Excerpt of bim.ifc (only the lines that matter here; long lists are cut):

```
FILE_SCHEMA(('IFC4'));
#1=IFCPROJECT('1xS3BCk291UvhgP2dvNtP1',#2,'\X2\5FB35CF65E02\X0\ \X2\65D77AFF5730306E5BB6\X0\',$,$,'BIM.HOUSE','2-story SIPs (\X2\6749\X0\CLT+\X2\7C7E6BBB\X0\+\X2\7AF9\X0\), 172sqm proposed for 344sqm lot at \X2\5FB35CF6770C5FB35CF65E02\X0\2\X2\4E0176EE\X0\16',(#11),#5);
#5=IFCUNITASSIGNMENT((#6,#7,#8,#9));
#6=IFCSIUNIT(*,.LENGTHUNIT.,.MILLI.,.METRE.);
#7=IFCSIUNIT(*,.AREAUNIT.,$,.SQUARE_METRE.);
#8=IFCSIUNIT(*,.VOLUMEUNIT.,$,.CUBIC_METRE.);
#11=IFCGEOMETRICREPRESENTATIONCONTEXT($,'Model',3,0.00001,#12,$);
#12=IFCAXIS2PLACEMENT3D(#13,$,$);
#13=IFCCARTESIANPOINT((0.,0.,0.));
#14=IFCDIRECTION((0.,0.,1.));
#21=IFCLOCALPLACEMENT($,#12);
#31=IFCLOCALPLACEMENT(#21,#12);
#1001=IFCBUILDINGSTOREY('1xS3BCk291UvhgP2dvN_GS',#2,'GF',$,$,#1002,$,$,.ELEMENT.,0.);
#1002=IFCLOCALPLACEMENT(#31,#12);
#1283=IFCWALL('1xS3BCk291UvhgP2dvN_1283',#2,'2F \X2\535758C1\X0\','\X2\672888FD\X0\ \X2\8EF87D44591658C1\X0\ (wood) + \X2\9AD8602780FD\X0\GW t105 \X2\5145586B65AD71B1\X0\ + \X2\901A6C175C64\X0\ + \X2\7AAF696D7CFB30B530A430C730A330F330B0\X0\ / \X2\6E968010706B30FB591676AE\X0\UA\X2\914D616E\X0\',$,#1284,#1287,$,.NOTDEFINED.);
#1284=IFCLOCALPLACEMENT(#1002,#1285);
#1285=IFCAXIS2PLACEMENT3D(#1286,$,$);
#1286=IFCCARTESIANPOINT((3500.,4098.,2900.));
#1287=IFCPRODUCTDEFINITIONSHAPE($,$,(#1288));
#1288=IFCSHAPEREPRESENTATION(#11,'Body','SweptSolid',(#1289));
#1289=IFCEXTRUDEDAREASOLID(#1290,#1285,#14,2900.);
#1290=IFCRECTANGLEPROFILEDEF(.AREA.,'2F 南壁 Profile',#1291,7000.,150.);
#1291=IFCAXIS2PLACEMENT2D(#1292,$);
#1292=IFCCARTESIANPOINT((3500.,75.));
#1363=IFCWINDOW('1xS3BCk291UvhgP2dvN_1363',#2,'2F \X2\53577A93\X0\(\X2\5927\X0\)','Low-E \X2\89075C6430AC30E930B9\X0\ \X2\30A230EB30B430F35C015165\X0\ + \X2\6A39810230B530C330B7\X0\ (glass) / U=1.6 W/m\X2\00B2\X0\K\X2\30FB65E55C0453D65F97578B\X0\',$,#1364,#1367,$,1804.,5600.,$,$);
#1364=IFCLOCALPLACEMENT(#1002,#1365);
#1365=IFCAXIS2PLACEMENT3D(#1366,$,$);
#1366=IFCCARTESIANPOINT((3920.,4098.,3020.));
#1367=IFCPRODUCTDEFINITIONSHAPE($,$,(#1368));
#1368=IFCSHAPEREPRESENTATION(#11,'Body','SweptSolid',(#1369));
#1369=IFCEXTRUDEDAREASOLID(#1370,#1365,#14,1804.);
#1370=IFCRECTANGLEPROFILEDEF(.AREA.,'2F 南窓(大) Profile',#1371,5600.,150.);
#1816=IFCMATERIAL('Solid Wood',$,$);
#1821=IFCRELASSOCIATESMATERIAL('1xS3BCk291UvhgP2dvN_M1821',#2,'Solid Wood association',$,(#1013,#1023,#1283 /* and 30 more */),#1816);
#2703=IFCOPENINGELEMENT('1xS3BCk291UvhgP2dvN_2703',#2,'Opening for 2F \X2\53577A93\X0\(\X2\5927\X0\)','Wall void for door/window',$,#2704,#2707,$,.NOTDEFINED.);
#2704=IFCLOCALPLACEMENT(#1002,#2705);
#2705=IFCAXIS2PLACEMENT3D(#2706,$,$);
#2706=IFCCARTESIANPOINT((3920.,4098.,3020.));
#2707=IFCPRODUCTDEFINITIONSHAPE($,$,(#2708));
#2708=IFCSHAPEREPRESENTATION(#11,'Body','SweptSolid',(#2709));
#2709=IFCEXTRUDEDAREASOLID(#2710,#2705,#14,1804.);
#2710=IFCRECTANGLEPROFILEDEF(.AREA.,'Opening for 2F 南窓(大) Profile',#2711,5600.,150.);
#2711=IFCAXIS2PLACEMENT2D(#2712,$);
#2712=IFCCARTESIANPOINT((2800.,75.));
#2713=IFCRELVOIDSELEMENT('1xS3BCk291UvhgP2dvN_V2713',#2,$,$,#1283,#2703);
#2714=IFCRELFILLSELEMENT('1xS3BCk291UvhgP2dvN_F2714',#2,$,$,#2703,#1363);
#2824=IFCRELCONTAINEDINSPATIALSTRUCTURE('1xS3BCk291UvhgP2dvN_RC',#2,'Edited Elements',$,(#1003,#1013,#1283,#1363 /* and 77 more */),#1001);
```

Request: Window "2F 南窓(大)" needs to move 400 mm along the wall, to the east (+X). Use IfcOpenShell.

```python
import ifcopenshell
import ifcopenshell.api.geometry
import ifcopenshell.util.placement

model = ifcopenshell.open("bim.ifc")

window = model.by_guid("1xS3BCk291UvhgP2dvN_1363")
opening = window.FillsVoids[0].RelatingOpeningElement
wall = opening.VoidsElements[0].RelatingBuildingElement

wall_matrix = ifcopenshell.util.placement.get_local_placement(wall.ObjectPlacement)
shift = wall_matrix[:3, 0] * 400.0
before = ifcopenshell.util.placement.get_local_placement(window.ObjectPlacement)[:3, 3].copy()

# The window is not placed relative to its opening, so move both.
for product in (opening, window):
    matrix = ifcopenshell.util.placement.get_local_placement(product.ObjectPlacement)
    matrix[:3, 3] += shift
    ifcopenshell.api.geometry.edit_object_placement(model, product=product, matrix=matrix, is_si=False)

after = ifcopenshell.util.placement.get_local_placement(window.ObjectPlacement)[:3, 3]
print("window moved by", (after - before).round(3) + 0.0)

model.write("bim_v2.ifc")
```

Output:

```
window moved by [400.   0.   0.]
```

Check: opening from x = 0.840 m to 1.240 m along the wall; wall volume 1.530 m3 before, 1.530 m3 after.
